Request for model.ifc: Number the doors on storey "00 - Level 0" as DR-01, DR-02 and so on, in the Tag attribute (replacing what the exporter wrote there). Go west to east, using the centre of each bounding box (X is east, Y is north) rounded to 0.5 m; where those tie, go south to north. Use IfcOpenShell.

First a look at what the model holds.

```python
import ifcopenshell
import ifcopenshell.util.element
import ifcopenshell.util.placement

model = ifcopenshell.open("model.ifc")
print(model.schema)
storey = next(s for s in model.by_type("IfcBuildingStorey") if s.Name == "00 - Level 0")
doors = [e for e in ifcopenshell.util.element.get_decomposition(storey) if e.is_a("IfcDoor")]
for e in sorted(doors, key=lambda e: e.id()):
    origin = ifcopenshell.util.placement.get_local_placement(e.ObjectPlacement)[:3, 3]
    print(e.id(), e.Tag, e.Name, origin.round(2) + 0.0, sep=" | ")
```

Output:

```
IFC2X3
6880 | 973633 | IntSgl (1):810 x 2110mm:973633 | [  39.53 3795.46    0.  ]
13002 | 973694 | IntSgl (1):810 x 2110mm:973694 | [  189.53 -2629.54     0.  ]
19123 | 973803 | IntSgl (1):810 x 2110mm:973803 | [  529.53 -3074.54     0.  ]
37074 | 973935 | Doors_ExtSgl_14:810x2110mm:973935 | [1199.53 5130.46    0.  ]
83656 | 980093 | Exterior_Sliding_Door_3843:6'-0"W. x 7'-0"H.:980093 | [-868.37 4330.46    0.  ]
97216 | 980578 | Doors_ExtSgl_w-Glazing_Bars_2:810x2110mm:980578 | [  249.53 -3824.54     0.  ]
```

```python
import ifcopenshell
import ifcopenshell.geom
import ifcopenshell.util.element
import ifcopenshell.util.shape

model = ifcopenshell.open("model.ifc")
settings = ifcopenshell.geom.settings()
settings.set("use-world-coords", True)


def centre(element):
    shape = ifcopenshell.geom.create_shape(settings, element)
    return ifcopenshell.util.shape.get_bbox_centroid(shape.geometry)


storey = next(s for s in model.by_type("IfcBuildingStorey") if s.Name == "00 - Level 0")
doors = [e for e in ifcopenshell.util.element.get_decomposition(storey) if e.is_a("IfcDoor")]

# Insertion points can sit at a corner or the storey origin, so sort by the geometry (in metres).
centres = {e: centre(e) for e in doors}
doors.sort(key=lambda e: (round(centres[e][0] / 0.5), centres[e][1]))

for i, e in enumerate(doors, start=1):
    number = f"DR-{i:02d}"
    e.Tag = number
    print(e.id(), number)

model.write("model-out.ifc")
```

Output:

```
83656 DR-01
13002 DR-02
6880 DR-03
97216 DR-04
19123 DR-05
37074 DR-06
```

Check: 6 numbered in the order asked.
